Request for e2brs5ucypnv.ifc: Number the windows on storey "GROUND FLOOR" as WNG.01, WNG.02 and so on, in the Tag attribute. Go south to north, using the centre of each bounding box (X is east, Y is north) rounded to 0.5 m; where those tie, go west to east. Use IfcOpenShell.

First a look at what the model holds.

```python
import ifcopenshell
import ifcopenshell.util.element
import ifcopenshell.util.placement

model = ifcopenshell.open("e2brs5ucypnv.ifc")
print(model.schema)
storey = next(s for s in model.by_type("IfcBuildingStorey") if s.Name == "GROUND FLOOR")
windows = [e for e in ifcopenshell.util.element.get_decomposition(storey) if e.is_a("IfcWindow")]
for e in sorted(windows, key=lambda e: e.id()):
    origin = ifcopenshell.util.placement.get_local_placement(e.ObjectPlacement)[:3, 3]
    print(e.id(), e.Tag, e.Name, origin.round(2) + 0.0, sep=" | ")
```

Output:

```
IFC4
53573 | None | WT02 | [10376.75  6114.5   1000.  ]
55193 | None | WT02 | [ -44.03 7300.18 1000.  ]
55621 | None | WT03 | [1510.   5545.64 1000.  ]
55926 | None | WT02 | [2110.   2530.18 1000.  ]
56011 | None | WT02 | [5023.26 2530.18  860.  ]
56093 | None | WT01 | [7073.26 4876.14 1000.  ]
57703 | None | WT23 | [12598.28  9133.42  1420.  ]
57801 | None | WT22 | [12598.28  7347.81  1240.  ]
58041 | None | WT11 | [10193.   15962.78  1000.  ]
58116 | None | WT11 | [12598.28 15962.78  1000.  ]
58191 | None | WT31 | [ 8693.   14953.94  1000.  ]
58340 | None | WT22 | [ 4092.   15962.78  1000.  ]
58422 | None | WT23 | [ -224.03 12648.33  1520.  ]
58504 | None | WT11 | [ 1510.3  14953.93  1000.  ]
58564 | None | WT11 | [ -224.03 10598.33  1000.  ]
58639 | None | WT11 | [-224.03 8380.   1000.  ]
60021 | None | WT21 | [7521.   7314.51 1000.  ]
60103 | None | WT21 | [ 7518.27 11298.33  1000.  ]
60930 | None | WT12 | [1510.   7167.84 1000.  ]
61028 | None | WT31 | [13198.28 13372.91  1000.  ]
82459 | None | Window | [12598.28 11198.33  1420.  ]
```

```python
import ifcopenshell
import ifcopenshell.geom
import ifcopenshell.util.element
import ifcopenshell.util.shape

model = ifcopenshell.open("e2brs5ucypnv.ifc")
settings = ifcopenshell.geom.settings()
settings.set("use-world-coords", True)


def centre(element):
    shape = ifcopenshell.geom.create_shape(settings, element)
    return ifcopenshell.util.shape.get_bbox_centroid(shape.geometry)


storey = next(s for s in model.by_type("IfcBuildingStorey") if s.Name == "GROUND FLOOR")
windows = [e for e in ifcopenshell.util.element.get_decomposition(storey) if e.is_a("IfcWindow")]

# Insertion points can sit at a corner or the storey origin, so sort by the geometry (in metres).
centres = {e: centre(e) for e in windows}
windows.sort(key=lambda e: (round(centres[e][1] / 0.5), centres[e][0]))

for i, e in enumerate(windows, start=1):
    number = f"WNG.{i:02d}"
    e.Tag = number
    print(e.id(), number)

model.write("e2brs5ucypnv_edited.ifc")
```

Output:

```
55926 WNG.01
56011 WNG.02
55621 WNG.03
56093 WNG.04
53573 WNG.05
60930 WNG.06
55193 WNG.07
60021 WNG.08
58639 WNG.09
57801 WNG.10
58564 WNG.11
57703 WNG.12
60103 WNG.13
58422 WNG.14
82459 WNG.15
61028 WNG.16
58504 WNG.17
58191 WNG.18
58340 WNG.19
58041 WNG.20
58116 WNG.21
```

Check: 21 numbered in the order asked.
